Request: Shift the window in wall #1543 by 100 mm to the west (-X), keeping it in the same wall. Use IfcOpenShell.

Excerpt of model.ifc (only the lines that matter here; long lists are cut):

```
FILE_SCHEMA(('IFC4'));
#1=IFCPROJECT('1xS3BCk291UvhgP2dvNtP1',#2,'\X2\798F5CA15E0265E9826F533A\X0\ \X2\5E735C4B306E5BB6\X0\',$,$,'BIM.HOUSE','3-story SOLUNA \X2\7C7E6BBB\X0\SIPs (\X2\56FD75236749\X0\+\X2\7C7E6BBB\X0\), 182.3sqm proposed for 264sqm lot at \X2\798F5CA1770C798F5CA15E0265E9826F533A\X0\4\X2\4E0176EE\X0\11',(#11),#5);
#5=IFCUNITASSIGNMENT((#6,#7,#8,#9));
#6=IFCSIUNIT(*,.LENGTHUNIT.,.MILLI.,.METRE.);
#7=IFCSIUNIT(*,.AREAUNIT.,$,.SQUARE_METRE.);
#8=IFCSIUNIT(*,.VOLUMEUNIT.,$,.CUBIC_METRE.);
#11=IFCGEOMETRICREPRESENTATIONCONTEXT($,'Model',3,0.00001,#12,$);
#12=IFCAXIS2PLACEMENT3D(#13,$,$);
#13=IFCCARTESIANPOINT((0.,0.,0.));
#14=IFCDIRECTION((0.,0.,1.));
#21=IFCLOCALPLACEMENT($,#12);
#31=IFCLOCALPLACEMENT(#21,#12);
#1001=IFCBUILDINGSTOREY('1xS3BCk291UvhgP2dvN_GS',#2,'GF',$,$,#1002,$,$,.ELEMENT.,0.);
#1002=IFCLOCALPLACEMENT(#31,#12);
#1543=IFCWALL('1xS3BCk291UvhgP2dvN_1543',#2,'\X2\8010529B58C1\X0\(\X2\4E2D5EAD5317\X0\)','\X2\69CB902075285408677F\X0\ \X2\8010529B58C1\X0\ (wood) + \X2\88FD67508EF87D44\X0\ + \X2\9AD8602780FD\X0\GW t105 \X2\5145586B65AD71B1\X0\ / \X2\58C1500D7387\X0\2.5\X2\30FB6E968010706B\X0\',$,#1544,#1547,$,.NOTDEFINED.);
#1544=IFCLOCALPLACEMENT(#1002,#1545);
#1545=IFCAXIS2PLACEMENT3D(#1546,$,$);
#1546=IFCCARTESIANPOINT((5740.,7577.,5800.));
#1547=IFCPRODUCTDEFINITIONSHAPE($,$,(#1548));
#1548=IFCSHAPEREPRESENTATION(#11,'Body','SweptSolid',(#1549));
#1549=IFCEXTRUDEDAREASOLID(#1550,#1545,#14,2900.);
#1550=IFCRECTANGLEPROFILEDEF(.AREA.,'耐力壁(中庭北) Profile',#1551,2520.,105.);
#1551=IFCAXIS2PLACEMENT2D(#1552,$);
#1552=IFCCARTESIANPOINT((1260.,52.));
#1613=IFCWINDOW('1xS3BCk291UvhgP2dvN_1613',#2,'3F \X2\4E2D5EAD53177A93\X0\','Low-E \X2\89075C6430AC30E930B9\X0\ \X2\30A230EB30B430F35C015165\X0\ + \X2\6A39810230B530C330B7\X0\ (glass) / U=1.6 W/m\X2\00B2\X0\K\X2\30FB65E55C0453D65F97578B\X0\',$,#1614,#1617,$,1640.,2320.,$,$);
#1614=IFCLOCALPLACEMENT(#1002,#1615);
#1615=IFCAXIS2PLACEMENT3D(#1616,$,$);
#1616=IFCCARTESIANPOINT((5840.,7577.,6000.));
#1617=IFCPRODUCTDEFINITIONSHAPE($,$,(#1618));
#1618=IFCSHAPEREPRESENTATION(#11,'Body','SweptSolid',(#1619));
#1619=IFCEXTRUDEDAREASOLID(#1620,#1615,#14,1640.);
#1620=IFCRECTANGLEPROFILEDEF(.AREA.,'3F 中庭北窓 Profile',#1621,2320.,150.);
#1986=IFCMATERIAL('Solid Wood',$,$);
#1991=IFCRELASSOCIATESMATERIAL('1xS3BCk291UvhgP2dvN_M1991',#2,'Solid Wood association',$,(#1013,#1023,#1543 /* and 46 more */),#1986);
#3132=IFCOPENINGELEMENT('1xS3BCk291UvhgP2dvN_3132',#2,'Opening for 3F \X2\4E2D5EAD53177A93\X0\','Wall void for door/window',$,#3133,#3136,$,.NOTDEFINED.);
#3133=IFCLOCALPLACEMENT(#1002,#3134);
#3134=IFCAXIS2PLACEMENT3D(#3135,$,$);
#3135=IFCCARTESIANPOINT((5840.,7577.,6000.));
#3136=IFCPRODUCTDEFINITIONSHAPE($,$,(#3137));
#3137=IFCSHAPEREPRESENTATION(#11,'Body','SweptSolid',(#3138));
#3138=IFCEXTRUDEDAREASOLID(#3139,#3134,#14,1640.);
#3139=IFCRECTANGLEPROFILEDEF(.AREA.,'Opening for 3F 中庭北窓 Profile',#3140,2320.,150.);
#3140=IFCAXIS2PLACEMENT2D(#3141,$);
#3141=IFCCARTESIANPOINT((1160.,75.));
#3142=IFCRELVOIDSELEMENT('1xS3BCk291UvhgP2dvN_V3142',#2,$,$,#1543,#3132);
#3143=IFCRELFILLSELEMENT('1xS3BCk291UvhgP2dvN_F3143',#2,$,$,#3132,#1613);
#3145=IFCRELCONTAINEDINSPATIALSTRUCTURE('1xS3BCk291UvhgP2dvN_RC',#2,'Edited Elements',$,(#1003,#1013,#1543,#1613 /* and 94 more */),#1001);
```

```python
import ifcopenshell
import ifcopenshell.api.geometry
import ifcopenshell.util.placement
import ifcopenshell.util.unit

model = ifcopenshell.open("model.ifc")
unit_scale = ifcopenshell.util.unit.calculate_unit_scale(model)

window = model.by_guid("1xS3BCk291UvhgP2dvN_1613")
opening = window.FillsVoids[0].RelatingOpeningElement
wall = opening.VoidsElements[0].RelatingBuildingElement

wall_matrix = ifcopenshell.util.placement.get_local_placement(wall.ObjectPlacement)
shift = wall_matrix[:3, 0] * -0.1 / unit_scale
before = ifcopenshell.util.placement.get_local_placement(window.ObjectPlacement)[:3, 3].copy()

# The window is not placed relative to its opening, so move both.
for product in (opening, window):
    matrix = ifcopenshell.util.placement.get_local_placement(product.ObjectPlacement)
    matrix[:3, 3] += shift
    ifcopenshell.api.geometry.edit_object_placement(model, product=product, matrix=matrix, is_si=False)

after = ifcopenshell.util.placement.get_local_placement(window.ObjectPlacement)[:3, 3]
print("window moved by", (after - before).round(3) + 0.0)

model.write("model-out.ifc")
```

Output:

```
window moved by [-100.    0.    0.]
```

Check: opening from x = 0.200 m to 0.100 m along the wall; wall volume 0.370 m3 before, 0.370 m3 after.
